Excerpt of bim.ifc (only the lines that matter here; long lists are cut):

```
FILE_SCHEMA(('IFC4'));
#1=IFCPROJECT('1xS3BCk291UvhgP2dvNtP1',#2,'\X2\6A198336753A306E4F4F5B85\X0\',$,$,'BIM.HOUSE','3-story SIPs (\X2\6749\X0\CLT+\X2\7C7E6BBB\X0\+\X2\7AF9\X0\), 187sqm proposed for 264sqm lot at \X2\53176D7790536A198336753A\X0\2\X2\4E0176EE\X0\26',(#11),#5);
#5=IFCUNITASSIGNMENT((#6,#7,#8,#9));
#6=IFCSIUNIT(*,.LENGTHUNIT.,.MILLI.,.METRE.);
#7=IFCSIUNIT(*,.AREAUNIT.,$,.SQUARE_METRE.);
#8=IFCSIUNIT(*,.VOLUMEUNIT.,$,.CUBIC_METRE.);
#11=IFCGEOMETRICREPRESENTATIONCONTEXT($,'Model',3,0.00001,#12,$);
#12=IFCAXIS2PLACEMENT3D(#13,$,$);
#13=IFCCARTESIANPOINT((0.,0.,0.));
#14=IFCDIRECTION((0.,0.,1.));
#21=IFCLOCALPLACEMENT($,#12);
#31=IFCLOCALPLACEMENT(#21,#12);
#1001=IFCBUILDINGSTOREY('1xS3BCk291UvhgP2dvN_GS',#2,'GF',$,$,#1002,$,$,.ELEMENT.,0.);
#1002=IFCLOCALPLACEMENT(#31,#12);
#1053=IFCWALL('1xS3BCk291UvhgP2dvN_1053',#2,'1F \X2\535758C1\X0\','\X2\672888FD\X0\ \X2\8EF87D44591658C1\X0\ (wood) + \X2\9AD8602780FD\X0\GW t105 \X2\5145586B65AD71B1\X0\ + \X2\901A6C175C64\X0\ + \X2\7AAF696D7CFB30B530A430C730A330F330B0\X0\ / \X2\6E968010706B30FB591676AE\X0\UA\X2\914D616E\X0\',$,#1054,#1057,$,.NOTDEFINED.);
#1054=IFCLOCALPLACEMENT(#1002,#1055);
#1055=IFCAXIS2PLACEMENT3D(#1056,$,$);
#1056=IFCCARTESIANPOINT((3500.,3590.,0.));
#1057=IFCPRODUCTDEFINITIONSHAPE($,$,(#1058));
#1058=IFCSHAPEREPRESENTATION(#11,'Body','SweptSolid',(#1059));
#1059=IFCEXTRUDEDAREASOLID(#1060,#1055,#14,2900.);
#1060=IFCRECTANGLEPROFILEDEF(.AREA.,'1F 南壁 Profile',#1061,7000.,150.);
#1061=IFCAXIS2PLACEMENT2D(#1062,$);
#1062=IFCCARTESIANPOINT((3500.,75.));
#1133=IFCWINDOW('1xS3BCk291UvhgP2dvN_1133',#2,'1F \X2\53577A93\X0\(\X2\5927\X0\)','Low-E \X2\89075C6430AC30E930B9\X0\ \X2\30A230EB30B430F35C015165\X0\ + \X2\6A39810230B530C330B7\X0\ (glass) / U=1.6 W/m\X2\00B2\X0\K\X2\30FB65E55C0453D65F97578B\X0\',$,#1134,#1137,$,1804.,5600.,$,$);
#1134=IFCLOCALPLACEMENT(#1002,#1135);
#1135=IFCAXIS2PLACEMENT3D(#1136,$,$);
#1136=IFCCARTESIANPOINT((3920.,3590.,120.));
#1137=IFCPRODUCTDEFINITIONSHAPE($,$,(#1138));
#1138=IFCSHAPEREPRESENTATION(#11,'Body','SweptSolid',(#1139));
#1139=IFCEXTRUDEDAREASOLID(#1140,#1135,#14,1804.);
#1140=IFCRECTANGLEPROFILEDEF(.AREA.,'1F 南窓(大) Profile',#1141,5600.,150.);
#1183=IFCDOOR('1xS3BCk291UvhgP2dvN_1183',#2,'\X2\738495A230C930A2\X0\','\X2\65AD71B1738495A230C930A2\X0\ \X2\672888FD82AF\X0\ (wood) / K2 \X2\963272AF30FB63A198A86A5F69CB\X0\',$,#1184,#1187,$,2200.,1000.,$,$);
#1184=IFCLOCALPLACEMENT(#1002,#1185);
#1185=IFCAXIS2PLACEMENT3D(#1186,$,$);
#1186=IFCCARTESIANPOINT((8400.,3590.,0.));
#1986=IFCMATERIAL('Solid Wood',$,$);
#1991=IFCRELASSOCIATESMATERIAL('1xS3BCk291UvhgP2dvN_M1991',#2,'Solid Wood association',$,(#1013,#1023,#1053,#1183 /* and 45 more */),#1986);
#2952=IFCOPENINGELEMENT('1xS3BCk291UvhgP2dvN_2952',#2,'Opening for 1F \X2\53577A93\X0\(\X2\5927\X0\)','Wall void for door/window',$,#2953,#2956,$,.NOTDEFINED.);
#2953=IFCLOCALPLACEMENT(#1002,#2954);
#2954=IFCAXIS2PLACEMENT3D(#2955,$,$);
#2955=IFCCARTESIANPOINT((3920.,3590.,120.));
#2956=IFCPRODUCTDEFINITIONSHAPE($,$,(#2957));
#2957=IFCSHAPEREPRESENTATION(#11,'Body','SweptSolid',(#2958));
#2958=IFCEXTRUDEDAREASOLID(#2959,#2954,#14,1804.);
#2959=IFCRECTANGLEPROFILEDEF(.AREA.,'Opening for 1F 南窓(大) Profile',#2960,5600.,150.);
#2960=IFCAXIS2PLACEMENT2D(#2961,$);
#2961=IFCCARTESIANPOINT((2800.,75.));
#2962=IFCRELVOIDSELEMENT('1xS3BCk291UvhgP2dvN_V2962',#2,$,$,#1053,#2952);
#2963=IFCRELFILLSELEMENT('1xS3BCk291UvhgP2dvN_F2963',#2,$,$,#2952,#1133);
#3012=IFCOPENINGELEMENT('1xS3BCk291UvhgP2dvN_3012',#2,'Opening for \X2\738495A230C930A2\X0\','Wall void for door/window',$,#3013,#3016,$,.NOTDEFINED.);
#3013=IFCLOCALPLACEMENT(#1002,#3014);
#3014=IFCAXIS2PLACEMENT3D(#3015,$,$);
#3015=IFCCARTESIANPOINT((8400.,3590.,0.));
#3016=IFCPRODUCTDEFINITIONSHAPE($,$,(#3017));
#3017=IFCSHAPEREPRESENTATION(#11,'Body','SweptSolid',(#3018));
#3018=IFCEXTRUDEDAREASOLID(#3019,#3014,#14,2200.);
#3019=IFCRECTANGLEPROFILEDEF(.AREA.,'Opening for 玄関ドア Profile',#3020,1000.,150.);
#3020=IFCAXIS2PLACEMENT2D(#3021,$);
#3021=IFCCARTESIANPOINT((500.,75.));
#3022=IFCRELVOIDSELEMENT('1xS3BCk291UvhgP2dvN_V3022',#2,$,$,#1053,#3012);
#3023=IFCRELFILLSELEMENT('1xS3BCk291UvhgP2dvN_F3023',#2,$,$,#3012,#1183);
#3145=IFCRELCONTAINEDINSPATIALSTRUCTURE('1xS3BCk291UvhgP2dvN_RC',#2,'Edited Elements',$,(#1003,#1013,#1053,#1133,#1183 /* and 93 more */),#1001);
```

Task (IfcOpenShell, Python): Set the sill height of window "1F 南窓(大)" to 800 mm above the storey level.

```python
import numpy as np
import ifcopenshell
import ifcopenshell.api.geometry
import ifcopenshell.geom
import ifcopenshell.util.element
import ifcopenshell.util.placement
import ifcopenshell.util.shape
import ifcopenshell.util.unit

model = ifcopenshell.open("bim.ifc")
unit_scale = ifcopenshell.util.unit.calculate_unit_scale(model)

window = model.by_guid("1xS3BCk291UvhgP2dvN_1133")
opening = window.FillsVoids[0].RelatingOpeningElement
storey = ifcopenshell.util.element.get_container(window, ifc_class="IfcBuildingStorey")
level = ifcopenshell.util.placement.get_local_placement(storey.ObjectPlacement)[2, 3]

# The opening's origin need not be at the sill, so measure its lowest point.
shape = ifcopenshell.geom.create_shape(ifcopenshell.geom.settings(), opening)
bottom = ifcopenshell.util.shape.get_shape_bottom_elevation(shape, shape.geometry) / unit_scale
dz = level + 0.8 / unit_scale - bottom

shift = np.array([0.0, 0.0, dz])
# The window is not placed relative to its opening, so move both.
for product in (opening, window):
    matrix = ifcopenshell.util.placement.get_local_placement(product.ObjectPlacement)
    matrix[:3, 3] += shift
    ifcopenshell.api.geometry.edit_object_placement(model, product=product, matrix=matrix, is_si=False)

print(f"moved by {dz * unit_scale:+.3f} m")

model.write("bim_rev.ifc")
```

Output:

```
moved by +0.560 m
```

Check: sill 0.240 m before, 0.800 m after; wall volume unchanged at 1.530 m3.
